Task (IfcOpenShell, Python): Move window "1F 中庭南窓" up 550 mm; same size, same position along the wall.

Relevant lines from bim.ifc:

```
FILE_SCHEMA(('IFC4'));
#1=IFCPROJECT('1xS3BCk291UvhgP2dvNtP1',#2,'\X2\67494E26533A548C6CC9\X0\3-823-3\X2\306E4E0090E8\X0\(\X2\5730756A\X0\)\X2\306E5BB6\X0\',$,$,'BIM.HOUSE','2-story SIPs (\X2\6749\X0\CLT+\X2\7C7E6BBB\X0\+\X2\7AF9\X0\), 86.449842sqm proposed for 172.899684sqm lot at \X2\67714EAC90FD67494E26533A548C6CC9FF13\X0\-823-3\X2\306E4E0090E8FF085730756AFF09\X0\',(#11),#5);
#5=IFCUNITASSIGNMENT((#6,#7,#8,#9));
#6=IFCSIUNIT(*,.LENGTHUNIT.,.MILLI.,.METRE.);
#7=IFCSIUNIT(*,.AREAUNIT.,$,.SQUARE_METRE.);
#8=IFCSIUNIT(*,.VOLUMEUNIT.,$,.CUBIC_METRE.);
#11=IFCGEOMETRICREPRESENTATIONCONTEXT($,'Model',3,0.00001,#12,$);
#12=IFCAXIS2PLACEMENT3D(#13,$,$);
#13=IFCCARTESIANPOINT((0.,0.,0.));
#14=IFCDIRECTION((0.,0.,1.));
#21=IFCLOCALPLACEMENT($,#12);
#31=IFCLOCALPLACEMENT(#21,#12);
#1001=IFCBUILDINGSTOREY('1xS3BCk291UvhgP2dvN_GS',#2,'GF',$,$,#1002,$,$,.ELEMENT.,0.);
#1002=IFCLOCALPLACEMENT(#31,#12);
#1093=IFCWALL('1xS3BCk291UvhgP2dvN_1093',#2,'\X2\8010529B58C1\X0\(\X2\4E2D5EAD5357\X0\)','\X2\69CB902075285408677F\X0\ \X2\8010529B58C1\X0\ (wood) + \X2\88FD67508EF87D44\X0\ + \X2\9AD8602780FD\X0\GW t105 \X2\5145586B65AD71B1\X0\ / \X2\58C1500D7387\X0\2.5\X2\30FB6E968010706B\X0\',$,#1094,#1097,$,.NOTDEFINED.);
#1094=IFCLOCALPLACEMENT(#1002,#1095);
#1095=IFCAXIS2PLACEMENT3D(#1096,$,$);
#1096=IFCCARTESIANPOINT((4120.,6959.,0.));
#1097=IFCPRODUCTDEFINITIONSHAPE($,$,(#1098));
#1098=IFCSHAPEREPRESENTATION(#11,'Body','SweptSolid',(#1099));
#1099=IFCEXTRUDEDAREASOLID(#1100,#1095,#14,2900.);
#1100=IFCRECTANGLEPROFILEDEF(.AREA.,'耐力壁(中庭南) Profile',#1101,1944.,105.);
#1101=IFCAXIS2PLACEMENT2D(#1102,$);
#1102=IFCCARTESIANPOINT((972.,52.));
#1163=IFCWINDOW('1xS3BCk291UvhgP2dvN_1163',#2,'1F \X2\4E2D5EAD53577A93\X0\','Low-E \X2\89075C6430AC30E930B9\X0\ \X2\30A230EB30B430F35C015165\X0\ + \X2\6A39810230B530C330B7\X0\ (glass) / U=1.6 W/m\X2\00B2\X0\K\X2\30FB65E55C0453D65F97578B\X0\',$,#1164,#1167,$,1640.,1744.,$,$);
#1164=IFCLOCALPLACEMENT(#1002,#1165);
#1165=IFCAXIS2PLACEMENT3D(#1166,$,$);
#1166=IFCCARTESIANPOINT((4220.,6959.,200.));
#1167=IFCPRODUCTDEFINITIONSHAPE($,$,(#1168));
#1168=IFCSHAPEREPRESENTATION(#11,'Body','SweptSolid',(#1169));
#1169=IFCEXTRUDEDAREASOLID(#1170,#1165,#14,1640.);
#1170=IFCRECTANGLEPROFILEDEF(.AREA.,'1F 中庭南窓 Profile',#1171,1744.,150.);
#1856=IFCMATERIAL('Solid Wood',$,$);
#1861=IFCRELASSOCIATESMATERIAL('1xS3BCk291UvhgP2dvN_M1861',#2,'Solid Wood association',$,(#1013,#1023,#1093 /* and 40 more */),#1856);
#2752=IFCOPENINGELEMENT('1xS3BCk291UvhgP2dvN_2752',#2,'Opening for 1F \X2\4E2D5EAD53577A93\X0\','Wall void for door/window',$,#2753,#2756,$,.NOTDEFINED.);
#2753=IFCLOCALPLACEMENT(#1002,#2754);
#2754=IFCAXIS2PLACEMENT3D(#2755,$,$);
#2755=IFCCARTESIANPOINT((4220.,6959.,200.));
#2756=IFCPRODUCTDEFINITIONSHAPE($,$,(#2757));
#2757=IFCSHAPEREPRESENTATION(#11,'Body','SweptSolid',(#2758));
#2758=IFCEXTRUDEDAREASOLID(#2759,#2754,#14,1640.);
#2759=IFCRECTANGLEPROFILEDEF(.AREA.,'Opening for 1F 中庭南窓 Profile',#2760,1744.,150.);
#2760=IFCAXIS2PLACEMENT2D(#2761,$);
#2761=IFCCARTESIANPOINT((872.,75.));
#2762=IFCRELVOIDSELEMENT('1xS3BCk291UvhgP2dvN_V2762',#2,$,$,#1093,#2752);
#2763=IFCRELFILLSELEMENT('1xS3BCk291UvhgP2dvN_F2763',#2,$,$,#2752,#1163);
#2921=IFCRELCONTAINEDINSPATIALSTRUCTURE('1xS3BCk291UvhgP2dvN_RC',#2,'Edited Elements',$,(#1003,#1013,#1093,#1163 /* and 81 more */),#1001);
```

```python
import numpy as np
import ifcopenshell
import ifcopenshell.api.geometry
import ifcopenshell.util.placement
import ifcopenshell.util.unit

model = ifcopenshell.open("bim.ifc")
unit_scale = ifcopenshell.util.unit.calculate_unit_scale(model)

window = model.by_guid("1xS3BCk291UvhgP2dvN_1163")
opening = window.FillsVoids[0].RelatingOpeningElement
dz = 0.55 / unit_scale

shift = np.array([0.0, 0.0, dz])
# The window is not placed relative to its opening, so move both.
for product in (opening, window):
    matrix = ifcopenshell.util.placement.get_local_placement(product.ObjectPlacement)
    matrix[:3, 3] += shift
    ifcopenshell.api.geometry.edit_object_placement(model, product=product, matrix=matrix, is_si=False)

print(f"moved by {dz * unit_scale:+.3f} m")

model.write("bim-out.ifc")
```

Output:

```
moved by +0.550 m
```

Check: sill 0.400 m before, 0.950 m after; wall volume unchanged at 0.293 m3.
